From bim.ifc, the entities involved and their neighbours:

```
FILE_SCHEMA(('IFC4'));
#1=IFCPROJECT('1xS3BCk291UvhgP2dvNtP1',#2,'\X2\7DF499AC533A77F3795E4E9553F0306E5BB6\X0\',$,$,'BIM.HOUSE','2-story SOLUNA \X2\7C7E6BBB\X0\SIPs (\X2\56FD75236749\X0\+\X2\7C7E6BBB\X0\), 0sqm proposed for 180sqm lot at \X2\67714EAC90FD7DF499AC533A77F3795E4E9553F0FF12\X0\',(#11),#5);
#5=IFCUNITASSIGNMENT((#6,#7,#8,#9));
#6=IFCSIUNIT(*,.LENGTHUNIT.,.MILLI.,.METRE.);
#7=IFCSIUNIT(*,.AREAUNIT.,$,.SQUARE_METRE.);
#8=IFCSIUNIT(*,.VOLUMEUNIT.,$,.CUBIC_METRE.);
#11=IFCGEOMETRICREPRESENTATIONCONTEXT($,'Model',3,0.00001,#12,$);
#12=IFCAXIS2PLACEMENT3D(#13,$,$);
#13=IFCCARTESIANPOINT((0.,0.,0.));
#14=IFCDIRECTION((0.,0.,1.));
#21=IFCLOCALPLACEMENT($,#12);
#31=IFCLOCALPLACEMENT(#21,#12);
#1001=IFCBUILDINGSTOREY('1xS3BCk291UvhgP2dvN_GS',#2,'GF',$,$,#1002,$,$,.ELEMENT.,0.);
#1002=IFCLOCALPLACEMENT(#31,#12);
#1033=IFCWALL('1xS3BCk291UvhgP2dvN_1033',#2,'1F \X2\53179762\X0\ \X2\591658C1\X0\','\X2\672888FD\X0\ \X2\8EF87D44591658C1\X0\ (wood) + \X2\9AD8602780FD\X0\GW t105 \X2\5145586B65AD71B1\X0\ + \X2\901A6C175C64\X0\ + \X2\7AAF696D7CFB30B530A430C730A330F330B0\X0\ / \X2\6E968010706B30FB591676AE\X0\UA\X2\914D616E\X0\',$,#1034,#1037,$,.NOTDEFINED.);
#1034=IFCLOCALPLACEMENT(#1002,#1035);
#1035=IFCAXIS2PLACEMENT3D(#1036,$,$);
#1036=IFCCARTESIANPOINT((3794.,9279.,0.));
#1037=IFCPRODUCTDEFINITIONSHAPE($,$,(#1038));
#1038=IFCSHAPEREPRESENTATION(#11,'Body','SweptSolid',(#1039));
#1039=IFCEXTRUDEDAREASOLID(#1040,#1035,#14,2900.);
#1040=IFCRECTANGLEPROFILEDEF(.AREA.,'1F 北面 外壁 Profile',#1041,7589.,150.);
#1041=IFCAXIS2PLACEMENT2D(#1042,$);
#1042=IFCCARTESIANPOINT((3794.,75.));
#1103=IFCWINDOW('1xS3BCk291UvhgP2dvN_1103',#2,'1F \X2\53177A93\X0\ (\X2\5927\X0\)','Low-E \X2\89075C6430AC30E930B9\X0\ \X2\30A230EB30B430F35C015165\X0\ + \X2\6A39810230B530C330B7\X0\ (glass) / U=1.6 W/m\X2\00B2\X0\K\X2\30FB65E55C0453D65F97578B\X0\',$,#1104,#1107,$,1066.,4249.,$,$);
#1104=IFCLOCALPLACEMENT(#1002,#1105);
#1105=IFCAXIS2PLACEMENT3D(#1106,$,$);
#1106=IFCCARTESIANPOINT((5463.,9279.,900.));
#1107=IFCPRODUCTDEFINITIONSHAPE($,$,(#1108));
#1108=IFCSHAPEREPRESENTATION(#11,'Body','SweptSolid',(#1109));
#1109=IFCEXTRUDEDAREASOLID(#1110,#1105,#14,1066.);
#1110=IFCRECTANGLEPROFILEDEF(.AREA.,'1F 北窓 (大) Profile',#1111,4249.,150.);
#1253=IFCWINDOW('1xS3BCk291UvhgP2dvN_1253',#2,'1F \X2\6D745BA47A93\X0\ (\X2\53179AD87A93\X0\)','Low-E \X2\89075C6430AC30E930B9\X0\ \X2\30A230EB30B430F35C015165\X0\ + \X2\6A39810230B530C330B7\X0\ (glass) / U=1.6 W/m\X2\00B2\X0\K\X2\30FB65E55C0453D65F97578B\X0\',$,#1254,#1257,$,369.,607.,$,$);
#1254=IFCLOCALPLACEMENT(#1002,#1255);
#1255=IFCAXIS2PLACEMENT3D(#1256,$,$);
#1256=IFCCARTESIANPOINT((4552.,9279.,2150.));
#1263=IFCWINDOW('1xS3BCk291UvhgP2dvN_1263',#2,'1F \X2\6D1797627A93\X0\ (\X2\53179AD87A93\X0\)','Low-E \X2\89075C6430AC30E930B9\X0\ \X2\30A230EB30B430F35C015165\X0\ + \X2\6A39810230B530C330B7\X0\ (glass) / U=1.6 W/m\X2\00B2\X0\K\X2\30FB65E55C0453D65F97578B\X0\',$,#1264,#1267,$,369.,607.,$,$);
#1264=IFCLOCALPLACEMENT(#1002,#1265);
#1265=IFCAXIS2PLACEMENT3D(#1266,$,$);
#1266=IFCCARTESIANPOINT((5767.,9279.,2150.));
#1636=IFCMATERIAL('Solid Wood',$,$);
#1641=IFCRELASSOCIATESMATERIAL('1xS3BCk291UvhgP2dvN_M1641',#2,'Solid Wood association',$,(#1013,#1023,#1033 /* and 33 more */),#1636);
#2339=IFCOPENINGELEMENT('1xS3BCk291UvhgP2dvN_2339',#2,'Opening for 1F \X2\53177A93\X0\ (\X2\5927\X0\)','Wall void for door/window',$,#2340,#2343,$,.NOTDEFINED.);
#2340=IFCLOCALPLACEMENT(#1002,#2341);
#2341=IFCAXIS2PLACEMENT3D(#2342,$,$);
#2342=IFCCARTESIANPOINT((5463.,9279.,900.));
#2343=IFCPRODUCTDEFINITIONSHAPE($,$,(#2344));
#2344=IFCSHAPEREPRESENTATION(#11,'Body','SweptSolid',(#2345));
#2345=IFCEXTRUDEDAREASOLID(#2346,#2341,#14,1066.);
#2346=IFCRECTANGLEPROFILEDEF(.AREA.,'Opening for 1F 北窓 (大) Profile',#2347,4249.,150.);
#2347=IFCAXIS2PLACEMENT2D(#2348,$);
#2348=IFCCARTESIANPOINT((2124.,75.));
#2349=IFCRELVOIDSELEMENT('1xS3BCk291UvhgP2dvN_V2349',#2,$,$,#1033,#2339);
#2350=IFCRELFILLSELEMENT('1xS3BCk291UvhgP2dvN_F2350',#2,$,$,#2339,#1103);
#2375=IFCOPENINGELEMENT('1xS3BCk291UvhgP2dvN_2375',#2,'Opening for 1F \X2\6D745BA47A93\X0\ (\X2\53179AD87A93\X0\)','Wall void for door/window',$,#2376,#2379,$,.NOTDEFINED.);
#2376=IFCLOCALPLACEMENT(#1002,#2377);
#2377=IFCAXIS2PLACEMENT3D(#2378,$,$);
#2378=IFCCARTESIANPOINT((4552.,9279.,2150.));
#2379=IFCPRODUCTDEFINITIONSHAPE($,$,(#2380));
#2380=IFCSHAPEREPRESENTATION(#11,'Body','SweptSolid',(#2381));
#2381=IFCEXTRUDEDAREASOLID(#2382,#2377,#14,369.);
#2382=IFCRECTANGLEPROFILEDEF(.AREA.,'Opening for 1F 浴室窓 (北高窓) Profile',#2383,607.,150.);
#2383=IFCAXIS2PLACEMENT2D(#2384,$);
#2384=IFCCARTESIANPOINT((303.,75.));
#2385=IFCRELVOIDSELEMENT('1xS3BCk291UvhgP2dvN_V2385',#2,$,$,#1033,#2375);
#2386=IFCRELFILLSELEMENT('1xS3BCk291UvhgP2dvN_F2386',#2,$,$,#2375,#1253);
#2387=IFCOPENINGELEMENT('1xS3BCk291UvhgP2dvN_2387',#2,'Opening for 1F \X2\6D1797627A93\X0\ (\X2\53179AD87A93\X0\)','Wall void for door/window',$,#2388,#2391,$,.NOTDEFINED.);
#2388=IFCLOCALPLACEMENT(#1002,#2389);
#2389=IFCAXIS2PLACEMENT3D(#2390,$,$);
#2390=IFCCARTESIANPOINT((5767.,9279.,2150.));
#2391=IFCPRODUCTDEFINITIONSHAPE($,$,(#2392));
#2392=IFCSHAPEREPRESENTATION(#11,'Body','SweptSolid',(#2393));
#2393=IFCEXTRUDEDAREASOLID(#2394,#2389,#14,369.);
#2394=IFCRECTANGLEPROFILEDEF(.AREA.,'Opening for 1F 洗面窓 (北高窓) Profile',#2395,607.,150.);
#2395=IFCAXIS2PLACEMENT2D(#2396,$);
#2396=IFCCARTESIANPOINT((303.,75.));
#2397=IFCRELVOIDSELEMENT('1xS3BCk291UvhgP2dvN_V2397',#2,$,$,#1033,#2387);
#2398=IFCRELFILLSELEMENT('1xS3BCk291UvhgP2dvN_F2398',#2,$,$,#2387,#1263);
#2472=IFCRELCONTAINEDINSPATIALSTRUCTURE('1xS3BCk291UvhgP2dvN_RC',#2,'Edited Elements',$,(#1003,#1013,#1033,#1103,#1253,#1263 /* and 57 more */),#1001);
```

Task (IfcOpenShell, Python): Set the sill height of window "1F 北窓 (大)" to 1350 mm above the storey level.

```python
import numpy as np
import ifcopenshell
import ifcopenshell.api.geometry
import ifcopenshell.geom
import ifcopenshell.util.element
import ifcopenshell.util.placement
import ifcopenshell.util.shape
import ifcopenshell.util.unit

model = ifcopenshell.open("bim.ifc")
unit_scale = ifcopenshell.util.unit.calculate_unit_scale(model)

window = model.by_guid("1xS3BCk291UvhgP2dvN_1103")
opening = window.FillsVoids[0].RelatingOpeningElement
storey = ifcopenshell.util.element.get_container(window, ifc_class="IfcBuildingStorey")
level = ifcopenshell.util.placement.get_local_placement(storey.ObjectPlacement)[2, 3]

# The opening's origin need not be at the sill, so measure its lowest point.
shape = ifcopenshell.geom.create_shape(ifcopenshell.geom.settings(), opening)
bottom = ifcopenshell.util.shape.get_shape_bottom_elevation(shape, shape.geometry) / unit_scale
dz = level + 1.35 / unit_scale - bottom

shift = np.array([0.0, 0.0, dz])
# The window is not placed relative to its opening, so move both.
for product in (opening, window):
    matrix = ifcopenshell.util.placement.get_local_placement(product.ObjectPlacement)
    matrix[:3, 3] += shift
    ifcopenshell.api.geometry.edit_object_placement(model, product=product, matrix=matrix, is_si=False)

print(f"moved by {dz * unit_scale:+.3f} m")

model.write("bim_rev.ifc")
```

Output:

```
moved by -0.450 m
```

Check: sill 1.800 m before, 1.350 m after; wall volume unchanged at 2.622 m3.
